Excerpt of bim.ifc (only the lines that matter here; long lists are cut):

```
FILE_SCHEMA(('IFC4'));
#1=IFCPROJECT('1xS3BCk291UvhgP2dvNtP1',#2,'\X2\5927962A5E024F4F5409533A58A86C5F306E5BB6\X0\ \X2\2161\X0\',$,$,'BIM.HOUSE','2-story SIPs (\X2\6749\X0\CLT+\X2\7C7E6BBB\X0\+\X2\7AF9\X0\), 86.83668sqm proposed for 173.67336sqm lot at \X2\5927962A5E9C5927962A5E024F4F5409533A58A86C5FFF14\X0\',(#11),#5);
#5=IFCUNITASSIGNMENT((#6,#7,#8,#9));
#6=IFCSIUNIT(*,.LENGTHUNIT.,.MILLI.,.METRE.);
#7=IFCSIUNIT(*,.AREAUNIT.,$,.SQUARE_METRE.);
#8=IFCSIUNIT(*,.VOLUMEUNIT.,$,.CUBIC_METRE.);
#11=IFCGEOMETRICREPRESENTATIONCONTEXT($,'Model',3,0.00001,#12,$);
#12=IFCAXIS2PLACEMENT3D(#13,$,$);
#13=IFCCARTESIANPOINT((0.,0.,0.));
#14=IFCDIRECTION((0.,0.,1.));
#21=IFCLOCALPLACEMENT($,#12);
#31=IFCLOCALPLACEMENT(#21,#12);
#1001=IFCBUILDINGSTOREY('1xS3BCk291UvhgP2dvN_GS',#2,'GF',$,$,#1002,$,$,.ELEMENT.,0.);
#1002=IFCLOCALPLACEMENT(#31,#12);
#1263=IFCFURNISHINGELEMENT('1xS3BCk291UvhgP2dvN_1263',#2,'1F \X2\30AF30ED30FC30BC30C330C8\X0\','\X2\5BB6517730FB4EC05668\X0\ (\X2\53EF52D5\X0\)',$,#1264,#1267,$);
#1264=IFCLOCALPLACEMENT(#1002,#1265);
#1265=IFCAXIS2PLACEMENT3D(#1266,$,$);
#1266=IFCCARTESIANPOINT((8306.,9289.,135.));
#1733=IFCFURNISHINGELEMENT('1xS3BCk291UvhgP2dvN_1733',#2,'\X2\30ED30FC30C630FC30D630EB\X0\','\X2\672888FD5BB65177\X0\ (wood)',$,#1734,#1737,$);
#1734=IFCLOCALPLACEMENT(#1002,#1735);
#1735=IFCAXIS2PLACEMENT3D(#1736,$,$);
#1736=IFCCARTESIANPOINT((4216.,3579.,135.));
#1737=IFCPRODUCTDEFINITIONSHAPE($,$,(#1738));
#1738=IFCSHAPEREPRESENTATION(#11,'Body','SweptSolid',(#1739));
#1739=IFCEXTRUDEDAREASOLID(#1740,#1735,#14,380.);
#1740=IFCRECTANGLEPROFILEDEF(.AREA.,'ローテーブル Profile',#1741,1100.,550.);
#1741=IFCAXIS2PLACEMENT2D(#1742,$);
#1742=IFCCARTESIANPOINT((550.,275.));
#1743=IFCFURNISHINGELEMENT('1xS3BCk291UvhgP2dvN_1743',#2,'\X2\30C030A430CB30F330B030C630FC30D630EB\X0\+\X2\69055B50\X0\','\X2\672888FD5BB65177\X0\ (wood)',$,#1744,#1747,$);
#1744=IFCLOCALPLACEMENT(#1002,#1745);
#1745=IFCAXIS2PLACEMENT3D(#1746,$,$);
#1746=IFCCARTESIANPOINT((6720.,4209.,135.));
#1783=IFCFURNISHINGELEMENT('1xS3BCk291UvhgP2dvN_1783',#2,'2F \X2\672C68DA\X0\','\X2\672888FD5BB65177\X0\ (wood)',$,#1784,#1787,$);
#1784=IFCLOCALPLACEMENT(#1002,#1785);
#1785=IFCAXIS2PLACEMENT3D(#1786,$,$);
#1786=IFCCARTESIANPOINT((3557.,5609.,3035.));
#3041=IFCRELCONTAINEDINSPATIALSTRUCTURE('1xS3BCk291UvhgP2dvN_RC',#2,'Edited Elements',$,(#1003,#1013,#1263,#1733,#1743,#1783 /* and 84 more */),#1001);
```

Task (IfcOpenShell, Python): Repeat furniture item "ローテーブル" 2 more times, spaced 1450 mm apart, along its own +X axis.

```python
import ifcopenshell
import ifcopenshell.api.geometry
import ifcopenshell.api.root
import ifcopenshell.util.element
import ifcopenshell.util.placement

model = ifcopenshell.open("bim.ifc")


def reuse_history(source, copy):
    """copy_class also copies each property set's owner history, people and application; keep the originals."""
    for rel in copy.IsDefinedBy:
        if rel.is_a("IfcRelDefinesByProperties") and (history := rel.RelatingPropertyDefinition.OwnerHistory):
            rel.RelatingPropertyDefinition.OwnerHistory = source.OwnerHistory
            ifcopenshell.util.element.remove_deep2(model, history)


source = model.by_id(1733)
base = ifcopenshell.util.placement.get_local_placement(source.ObjectPlacement)
step = base[:3, 0] * 1450.0

for i in range(1, 3):
    copy = ifcopenshell.api.root.copy_class(model, product=source)
    copy.Representation = ifcopenshell.util.element.copy_deep(
        model, source.Representation, exclude=["IfcGeometricRepresentationContext", "IfcRepresentationMap"]
    )
    reuse_history(source, copy)
    matrix = base.copy()
    matrix[:3, 3] += i * step
    print("added at", matrix[:3, 3].round(3) + 0.0)
    ifcopenshell.api.geometry.edit_object_placement(model, product=copy, matrix=matrix, is_si=False)

model.write("bim_edited.ifc")
```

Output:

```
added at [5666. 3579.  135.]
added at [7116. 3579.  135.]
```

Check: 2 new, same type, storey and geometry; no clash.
